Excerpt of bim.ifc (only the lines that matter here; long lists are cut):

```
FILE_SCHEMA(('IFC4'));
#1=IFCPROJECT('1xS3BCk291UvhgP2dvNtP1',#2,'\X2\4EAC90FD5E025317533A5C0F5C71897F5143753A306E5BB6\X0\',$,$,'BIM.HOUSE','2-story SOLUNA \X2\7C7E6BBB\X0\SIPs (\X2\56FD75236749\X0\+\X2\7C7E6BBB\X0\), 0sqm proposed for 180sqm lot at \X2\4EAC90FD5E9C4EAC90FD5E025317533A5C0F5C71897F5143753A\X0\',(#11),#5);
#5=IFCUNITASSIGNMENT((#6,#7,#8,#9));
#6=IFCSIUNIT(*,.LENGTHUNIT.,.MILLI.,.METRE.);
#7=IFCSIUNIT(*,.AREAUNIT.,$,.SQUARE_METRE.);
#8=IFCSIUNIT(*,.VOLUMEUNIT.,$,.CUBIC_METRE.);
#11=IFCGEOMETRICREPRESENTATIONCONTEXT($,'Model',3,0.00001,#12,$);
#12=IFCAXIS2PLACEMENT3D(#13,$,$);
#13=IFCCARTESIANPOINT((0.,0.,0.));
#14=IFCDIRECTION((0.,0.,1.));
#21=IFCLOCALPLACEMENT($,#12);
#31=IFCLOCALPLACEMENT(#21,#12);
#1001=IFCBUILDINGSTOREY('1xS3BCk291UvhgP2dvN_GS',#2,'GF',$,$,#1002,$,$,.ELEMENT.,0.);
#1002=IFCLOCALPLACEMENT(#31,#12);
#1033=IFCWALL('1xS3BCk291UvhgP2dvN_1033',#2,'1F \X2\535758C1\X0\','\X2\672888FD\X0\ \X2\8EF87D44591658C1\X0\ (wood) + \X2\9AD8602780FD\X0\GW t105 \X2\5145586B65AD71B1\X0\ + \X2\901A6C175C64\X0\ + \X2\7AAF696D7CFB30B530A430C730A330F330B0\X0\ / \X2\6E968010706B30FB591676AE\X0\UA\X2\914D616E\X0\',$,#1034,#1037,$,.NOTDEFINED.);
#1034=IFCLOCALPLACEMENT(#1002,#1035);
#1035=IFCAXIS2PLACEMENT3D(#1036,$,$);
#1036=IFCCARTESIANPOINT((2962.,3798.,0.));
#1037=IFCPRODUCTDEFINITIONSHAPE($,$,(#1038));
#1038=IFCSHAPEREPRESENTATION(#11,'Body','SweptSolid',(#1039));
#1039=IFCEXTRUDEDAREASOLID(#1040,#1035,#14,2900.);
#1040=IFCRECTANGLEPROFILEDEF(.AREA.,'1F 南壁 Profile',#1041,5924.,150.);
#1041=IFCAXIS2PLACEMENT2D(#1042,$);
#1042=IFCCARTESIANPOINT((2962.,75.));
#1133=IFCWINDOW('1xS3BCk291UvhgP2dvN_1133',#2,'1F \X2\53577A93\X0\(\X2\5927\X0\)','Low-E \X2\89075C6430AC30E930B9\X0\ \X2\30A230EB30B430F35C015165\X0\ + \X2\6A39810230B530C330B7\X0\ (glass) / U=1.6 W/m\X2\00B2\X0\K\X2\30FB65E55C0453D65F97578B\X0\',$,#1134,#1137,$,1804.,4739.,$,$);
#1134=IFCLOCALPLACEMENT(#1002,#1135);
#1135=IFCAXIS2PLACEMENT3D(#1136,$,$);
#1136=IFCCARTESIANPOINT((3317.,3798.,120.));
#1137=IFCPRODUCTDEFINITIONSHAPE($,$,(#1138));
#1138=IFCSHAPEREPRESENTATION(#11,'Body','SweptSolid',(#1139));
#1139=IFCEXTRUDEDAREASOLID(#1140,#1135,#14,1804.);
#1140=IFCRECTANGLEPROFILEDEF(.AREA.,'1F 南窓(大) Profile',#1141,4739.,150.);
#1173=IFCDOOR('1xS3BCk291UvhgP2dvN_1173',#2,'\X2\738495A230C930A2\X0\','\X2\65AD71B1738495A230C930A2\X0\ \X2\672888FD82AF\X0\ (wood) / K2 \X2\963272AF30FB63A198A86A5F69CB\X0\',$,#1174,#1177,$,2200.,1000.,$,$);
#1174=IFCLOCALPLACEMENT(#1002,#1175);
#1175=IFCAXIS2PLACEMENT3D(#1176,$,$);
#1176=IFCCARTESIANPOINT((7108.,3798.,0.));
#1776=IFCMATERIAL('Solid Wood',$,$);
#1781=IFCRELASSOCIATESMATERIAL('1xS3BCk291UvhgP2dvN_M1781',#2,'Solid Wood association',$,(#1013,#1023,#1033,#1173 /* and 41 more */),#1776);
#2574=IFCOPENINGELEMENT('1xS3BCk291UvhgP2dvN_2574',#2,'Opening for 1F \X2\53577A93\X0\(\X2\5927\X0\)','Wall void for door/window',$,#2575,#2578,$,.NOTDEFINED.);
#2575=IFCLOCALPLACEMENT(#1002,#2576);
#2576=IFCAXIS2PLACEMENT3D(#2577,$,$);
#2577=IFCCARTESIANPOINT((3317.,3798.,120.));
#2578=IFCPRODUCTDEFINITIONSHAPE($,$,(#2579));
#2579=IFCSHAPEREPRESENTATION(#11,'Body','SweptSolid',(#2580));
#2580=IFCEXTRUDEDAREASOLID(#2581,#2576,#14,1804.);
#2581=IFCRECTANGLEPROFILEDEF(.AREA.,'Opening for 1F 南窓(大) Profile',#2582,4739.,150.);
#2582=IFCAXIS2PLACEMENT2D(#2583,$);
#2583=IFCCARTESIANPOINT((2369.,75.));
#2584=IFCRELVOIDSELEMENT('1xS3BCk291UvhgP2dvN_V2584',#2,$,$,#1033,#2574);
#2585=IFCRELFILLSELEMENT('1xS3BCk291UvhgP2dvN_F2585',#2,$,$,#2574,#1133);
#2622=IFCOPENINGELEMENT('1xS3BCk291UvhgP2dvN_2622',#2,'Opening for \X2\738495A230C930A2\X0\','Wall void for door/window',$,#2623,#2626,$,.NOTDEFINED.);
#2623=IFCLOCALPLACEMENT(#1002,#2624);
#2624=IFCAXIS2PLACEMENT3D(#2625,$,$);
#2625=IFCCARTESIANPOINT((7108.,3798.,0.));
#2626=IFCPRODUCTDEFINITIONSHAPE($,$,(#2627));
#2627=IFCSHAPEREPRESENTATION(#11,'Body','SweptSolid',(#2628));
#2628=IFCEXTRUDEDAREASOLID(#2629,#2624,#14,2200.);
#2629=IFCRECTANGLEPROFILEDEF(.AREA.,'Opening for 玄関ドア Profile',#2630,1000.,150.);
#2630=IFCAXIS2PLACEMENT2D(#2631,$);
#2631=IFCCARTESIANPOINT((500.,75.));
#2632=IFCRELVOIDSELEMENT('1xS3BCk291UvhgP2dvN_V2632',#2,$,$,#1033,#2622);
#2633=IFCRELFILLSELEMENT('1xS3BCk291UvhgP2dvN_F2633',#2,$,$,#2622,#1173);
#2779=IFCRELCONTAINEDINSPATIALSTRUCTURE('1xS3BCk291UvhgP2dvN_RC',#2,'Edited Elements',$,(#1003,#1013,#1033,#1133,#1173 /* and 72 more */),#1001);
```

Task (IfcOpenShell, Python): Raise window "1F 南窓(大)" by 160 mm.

```python
import numpy as np
import ifcopenshell
import ifcopenshell.api.geometry
import ifcopenshell.util.placement
import ifcopenshell.util.unit

model = ifcopenshell.open("bim.ifc")
unit_scale = ifcopenshell.util.unit.calculate_unit_scale(model)

window = model.by_id(1133)
opening = window.FillsVoids[0].RelatingOpeningElement
dz = 0.16 / unit_scale

shift = np.array([0.0, 0.0, dz])
# The window is not placed relative to its opening, so move both.
for product in (opening, window):
    matrix = ifcopenshell.util.placement.get_local_placement(product.ObjectPlacement)
    matrix[:3, 3] += shift
    ifcopenshell.api.geometry.edit_object_placement(model, product=product, matrix=matrix, is_si=False)

print(f"moved by {dz * unit_scale:+.3f} m")

model.write("bim_edited.ifc")
```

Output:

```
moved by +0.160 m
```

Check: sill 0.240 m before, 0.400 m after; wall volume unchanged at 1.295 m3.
